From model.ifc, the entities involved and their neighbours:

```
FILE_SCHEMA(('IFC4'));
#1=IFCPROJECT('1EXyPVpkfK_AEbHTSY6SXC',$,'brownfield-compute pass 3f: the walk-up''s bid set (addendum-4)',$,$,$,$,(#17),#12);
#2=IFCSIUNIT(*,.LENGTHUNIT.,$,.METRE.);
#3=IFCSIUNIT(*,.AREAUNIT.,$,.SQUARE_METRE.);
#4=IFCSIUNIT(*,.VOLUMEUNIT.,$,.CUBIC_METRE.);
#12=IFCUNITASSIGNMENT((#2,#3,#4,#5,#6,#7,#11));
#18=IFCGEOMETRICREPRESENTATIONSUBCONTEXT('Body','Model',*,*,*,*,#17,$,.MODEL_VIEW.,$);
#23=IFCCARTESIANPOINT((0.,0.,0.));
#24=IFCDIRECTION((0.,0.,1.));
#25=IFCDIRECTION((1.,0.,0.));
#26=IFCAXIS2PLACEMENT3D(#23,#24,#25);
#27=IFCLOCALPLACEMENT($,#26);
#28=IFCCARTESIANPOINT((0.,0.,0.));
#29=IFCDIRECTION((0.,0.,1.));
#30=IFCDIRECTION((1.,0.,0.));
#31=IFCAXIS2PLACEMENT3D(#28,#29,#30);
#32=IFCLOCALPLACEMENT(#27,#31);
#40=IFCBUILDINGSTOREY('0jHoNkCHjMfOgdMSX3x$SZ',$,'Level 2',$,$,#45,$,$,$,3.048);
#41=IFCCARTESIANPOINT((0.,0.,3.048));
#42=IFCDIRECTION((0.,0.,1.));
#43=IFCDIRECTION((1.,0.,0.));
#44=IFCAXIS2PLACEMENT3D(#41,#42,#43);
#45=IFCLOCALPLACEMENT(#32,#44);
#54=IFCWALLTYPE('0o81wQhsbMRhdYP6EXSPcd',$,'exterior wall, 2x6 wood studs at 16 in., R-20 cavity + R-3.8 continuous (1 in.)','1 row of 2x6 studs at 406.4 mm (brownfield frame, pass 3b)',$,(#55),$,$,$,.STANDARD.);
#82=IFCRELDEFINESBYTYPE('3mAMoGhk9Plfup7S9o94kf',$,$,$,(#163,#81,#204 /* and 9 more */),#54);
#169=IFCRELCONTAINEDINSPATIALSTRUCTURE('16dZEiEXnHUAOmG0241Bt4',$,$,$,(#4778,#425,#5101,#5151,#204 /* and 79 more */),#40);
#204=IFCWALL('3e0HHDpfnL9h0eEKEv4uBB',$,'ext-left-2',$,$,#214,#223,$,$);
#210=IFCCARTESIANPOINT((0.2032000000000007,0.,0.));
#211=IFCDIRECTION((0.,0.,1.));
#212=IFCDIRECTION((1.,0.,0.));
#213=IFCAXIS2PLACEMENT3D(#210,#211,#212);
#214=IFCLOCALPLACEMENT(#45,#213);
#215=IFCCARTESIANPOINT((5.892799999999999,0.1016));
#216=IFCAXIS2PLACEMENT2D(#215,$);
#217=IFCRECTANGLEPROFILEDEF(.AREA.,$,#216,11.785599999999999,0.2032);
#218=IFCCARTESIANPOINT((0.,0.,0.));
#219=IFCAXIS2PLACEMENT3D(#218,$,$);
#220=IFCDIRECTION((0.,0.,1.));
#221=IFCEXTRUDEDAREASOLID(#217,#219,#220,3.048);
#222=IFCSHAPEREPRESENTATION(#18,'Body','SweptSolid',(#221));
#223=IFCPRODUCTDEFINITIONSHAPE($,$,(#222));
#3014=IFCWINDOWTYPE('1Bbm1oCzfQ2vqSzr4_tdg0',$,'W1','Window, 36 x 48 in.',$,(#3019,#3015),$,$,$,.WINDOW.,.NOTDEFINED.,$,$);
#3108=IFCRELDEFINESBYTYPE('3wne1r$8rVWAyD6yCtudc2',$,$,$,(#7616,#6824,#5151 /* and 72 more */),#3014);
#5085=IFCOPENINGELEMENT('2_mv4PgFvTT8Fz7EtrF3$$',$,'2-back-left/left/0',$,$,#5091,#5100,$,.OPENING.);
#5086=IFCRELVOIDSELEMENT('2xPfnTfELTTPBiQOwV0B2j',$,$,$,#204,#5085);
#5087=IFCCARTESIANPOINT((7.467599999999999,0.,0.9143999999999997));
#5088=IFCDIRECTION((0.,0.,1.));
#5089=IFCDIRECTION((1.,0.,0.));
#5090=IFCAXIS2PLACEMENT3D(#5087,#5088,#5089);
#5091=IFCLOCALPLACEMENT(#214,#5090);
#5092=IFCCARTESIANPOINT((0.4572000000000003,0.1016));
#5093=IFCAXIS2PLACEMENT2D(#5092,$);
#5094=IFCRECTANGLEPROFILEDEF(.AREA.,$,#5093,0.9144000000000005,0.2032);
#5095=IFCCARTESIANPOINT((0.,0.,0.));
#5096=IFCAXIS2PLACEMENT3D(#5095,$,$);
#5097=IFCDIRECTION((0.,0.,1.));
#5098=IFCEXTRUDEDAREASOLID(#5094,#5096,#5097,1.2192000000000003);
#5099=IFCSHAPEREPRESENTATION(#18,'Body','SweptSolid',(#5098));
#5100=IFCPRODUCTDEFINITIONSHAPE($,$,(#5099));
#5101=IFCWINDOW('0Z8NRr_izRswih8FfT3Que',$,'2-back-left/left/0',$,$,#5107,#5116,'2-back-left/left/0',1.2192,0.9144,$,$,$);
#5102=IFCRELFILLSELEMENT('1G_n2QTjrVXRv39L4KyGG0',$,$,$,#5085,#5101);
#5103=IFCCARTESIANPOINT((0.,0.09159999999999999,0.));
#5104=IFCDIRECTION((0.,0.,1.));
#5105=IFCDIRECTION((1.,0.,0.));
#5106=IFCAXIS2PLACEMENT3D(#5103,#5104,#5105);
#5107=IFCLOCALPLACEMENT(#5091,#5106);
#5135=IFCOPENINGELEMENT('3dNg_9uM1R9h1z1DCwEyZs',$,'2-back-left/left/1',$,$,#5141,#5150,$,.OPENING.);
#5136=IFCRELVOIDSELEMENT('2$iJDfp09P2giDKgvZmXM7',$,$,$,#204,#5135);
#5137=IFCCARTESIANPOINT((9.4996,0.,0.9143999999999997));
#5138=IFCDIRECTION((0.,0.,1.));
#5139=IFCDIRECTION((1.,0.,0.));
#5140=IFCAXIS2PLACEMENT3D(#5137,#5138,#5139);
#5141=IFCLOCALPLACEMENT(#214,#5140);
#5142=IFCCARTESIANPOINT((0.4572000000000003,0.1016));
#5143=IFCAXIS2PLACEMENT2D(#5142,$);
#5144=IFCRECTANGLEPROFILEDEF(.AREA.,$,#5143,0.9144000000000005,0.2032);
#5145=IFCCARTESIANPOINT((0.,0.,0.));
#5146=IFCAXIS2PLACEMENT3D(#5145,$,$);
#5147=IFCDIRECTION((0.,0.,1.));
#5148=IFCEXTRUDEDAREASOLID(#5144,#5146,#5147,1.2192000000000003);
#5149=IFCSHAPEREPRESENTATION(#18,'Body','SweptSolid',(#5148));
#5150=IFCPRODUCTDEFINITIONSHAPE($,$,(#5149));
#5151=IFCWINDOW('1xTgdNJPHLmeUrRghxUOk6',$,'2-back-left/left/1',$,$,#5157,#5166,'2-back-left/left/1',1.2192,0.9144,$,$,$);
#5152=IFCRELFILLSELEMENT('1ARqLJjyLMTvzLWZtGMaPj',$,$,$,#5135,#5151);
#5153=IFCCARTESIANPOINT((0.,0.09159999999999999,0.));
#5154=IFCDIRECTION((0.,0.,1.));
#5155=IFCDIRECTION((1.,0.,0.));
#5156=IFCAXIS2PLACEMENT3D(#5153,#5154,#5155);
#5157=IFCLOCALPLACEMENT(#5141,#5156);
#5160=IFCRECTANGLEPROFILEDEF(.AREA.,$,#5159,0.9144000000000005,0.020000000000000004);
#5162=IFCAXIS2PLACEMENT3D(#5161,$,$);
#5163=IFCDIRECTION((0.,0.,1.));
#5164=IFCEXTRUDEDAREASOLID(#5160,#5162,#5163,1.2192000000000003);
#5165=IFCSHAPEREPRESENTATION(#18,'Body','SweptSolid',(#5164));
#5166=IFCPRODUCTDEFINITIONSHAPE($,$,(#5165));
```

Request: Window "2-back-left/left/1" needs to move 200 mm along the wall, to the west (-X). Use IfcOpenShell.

```python
import ifcopenshell
import ifcopenshell.api.geometry
import ifcopenshell.util.placement
import ifcopenshell.util.unit

model = ifcopenshell.open("model.ifc")
unit_scale = ifcopenshell.util.unit.calculate_unit_scale(model)

window = model.by_guid("1xTgdNJPHLmeUrRghxUOk6")
opening = window.FillsVoids[0].RelatingOpeningElement
wall = opening.VoidsElements[0].RelatingBuildingElement

wall_matrix = ifcopenshell.util.placement.get_local_placement(wall.ObjectPlacement)
shift = wall_matrix[:3, 0] * -0.2 / unit_scale
before = ifcopenshell.util.placement.get_local_placement(window.ObjectPlacement)[:3, 3].copy()

# The window is placed relative to its opening, so it follows when the opening moves.
matrix = ifcopenshell.util.placement.get_local_placement(opening.ObjectPlacement)
matrix[:3, 3] += shift
ifcopenshell.api.geometry.edit_object_placement(
    model, product=opening, matrix=matrix, is_si=False, should_transform_children=True
)

after = ifcopenshell.util.placement.get_local_placement(window.ObjectPlacement)[:3, 3]
print("window moved by", (after - before).round(3) + 0.0)

model.write("model-out.ifc")
```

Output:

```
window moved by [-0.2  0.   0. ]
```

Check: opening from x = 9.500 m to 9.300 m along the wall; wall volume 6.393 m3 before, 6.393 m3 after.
